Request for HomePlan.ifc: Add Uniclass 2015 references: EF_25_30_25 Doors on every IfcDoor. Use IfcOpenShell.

First a look at what the model holds.

```python
import ifcopenshell

model = ifcopenshell.open("HomePlan.ifc")
print(model.schema)
print("classifications:", [c.Name for c in model.by_type("IfcClassification")])
for ifc_class in ("IfcDoor", "IfcRoof", "IfcStair", "IfcWall", "IfcWindow"):
    print(ifc_class, len(model.by_type(ifc_class)))
```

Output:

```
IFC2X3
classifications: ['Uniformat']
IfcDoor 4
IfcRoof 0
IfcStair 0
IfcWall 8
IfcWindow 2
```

```python
import ifcopenshell
import ifcopenshell.api.classification

model = ifcopenshell.open("HomePlan.ifc")

# IFC2X3 requires Source and Edition and has no link from the project to the system.
system = model.create_entity("IfcClassification", Source="NBS", Edition="2015", Name="Uniclass 2015")

codes = {
    "IfcDoor": ("EF_25_30_25", "Doors"),
}
for ifc_class, (code, name) in codes.items():
    products = model.by_type(ifc_class)
    ifcopenshell.api.classification.add_reference(
        model, products=products, classification=system, identification=code, name=name
    )
    print(code, len(products))

model.write("HomePlan_v2.ifc")
```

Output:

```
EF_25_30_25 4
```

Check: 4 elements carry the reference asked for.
